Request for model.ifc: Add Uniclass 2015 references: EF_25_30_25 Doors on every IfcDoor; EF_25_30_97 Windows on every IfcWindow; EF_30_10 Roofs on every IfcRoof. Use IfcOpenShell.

First a look at what the model holds.

```python
import ifcopenshell

model = ifcopenshell.open("model.ifc")
print(model.schema)
print("classifications:", [c.Name for c in model.by_type("IfcClassification")])
for ifc_class in ("IfcDoor", "IfcRoof", "IfcStair", "IfcWall", "IfcWindow"):
    print(ifc_class, len(model.by_type(ifc_class)))
```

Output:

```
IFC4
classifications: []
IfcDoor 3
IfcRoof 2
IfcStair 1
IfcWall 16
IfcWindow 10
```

```python
import ifcopenshell
import ifcopenshell.api.classification

model = ifcopenshell.open("model.ifc")

system = ifcopenshell.api.classification.add_classification(model, classification="Uniclass 2015")

codes = {
    "IfcDoor": ("EF_25_30_25", "Doors"),
    "IfcWindow": ("EF_25_30_97", "Windows"),
    "IfcRoof": ("EF_30_10", "Roofs"),
}
for ifc_class, (code, name) in codes.items():
    products = model.by_type(ifc_class)
    ifcopenshell.api.classification.add_reference(
        model, products=products, classification=system, identification=code, name=name
    )
    print(code, len(products))

model.write("model_edited.ifc")
```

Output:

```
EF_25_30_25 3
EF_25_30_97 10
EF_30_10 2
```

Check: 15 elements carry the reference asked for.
